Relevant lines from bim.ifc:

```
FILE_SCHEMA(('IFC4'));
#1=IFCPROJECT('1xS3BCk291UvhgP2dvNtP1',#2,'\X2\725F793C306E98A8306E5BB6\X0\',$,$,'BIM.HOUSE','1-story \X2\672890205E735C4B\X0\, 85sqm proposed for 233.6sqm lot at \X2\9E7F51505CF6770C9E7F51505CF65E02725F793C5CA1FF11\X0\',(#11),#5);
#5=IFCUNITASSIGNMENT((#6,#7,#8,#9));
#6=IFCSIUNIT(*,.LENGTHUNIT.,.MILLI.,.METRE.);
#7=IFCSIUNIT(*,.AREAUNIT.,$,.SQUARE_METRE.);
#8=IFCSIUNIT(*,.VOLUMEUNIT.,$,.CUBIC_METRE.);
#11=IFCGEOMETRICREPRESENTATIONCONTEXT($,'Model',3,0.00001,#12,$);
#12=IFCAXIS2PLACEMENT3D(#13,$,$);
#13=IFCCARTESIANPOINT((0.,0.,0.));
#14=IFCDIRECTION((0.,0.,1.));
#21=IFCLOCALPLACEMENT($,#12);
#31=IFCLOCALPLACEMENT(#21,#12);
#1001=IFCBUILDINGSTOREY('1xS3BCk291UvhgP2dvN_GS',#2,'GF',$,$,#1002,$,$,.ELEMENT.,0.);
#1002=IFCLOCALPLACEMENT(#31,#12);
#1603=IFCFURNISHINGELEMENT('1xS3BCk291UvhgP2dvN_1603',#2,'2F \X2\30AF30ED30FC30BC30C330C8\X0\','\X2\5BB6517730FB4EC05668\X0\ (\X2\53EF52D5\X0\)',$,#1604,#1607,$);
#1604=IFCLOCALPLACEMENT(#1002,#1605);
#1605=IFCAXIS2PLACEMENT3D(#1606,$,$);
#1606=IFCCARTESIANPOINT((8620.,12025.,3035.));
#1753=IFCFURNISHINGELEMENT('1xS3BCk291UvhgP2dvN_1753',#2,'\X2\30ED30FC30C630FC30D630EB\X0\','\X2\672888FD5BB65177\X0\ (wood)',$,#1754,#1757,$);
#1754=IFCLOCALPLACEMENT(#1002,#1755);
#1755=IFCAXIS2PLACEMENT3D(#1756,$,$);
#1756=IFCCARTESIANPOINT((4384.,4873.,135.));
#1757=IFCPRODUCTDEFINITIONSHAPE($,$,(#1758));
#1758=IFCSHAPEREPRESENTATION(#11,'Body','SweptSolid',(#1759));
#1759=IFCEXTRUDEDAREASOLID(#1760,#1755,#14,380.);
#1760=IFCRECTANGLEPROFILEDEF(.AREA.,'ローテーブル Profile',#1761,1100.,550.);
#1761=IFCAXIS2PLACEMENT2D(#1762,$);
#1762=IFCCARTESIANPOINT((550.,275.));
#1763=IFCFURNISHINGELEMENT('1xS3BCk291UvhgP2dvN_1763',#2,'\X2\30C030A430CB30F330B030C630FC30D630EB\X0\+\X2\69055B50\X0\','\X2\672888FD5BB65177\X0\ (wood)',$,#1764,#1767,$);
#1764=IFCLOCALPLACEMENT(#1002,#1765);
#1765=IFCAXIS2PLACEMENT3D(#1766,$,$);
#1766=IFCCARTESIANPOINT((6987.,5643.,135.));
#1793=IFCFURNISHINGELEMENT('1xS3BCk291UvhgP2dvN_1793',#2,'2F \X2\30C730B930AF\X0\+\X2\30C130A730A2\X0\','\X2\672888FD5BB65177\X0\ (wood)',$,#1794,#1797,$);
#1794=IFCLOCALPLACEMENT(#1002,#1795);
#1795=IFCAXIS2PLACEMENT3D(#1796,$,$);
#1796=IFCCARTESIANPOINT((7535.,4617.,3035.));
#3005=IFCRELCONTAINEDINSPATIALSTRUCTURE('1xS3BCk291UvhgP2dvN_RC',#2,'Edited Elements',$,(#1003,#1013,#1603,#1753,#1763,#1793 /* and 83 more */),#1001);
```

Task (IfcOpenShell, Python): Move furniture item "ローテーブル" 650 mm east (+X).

```python
import ifcopenshell
import ifcopenshell.api.geometry
import ifcopenshell.util.placement
import ifcopenshell.util.unit

model = ifcopenshell.open("bim.ifc")
unit_scale = ifcopenshell.util.unit.calculate_unit_scale(model)

item = model.by_id(1753)
matrix = ifcopenshell.util.placement.get_local_placement(item.ObjectPlacement)
matrix[0, 3] += 0.65 / unit_scale
ifcopenshell.api.geometry.edit_object_placement(model, product=item, matrix=matrix, is_si=False)

print(ifcopenshell.util.placement.get_local_placement(item.ObjectPlacement).round(3) + 0.0)

model.write("bim-out.ifc")
```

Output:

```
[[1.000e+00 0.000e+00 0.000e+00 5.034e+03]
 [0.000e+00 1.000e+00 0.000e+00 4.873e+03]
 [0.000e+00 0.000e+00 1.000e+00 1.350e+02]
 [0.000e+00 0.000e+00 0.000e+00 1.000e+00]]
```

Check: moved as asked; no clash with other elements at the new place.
